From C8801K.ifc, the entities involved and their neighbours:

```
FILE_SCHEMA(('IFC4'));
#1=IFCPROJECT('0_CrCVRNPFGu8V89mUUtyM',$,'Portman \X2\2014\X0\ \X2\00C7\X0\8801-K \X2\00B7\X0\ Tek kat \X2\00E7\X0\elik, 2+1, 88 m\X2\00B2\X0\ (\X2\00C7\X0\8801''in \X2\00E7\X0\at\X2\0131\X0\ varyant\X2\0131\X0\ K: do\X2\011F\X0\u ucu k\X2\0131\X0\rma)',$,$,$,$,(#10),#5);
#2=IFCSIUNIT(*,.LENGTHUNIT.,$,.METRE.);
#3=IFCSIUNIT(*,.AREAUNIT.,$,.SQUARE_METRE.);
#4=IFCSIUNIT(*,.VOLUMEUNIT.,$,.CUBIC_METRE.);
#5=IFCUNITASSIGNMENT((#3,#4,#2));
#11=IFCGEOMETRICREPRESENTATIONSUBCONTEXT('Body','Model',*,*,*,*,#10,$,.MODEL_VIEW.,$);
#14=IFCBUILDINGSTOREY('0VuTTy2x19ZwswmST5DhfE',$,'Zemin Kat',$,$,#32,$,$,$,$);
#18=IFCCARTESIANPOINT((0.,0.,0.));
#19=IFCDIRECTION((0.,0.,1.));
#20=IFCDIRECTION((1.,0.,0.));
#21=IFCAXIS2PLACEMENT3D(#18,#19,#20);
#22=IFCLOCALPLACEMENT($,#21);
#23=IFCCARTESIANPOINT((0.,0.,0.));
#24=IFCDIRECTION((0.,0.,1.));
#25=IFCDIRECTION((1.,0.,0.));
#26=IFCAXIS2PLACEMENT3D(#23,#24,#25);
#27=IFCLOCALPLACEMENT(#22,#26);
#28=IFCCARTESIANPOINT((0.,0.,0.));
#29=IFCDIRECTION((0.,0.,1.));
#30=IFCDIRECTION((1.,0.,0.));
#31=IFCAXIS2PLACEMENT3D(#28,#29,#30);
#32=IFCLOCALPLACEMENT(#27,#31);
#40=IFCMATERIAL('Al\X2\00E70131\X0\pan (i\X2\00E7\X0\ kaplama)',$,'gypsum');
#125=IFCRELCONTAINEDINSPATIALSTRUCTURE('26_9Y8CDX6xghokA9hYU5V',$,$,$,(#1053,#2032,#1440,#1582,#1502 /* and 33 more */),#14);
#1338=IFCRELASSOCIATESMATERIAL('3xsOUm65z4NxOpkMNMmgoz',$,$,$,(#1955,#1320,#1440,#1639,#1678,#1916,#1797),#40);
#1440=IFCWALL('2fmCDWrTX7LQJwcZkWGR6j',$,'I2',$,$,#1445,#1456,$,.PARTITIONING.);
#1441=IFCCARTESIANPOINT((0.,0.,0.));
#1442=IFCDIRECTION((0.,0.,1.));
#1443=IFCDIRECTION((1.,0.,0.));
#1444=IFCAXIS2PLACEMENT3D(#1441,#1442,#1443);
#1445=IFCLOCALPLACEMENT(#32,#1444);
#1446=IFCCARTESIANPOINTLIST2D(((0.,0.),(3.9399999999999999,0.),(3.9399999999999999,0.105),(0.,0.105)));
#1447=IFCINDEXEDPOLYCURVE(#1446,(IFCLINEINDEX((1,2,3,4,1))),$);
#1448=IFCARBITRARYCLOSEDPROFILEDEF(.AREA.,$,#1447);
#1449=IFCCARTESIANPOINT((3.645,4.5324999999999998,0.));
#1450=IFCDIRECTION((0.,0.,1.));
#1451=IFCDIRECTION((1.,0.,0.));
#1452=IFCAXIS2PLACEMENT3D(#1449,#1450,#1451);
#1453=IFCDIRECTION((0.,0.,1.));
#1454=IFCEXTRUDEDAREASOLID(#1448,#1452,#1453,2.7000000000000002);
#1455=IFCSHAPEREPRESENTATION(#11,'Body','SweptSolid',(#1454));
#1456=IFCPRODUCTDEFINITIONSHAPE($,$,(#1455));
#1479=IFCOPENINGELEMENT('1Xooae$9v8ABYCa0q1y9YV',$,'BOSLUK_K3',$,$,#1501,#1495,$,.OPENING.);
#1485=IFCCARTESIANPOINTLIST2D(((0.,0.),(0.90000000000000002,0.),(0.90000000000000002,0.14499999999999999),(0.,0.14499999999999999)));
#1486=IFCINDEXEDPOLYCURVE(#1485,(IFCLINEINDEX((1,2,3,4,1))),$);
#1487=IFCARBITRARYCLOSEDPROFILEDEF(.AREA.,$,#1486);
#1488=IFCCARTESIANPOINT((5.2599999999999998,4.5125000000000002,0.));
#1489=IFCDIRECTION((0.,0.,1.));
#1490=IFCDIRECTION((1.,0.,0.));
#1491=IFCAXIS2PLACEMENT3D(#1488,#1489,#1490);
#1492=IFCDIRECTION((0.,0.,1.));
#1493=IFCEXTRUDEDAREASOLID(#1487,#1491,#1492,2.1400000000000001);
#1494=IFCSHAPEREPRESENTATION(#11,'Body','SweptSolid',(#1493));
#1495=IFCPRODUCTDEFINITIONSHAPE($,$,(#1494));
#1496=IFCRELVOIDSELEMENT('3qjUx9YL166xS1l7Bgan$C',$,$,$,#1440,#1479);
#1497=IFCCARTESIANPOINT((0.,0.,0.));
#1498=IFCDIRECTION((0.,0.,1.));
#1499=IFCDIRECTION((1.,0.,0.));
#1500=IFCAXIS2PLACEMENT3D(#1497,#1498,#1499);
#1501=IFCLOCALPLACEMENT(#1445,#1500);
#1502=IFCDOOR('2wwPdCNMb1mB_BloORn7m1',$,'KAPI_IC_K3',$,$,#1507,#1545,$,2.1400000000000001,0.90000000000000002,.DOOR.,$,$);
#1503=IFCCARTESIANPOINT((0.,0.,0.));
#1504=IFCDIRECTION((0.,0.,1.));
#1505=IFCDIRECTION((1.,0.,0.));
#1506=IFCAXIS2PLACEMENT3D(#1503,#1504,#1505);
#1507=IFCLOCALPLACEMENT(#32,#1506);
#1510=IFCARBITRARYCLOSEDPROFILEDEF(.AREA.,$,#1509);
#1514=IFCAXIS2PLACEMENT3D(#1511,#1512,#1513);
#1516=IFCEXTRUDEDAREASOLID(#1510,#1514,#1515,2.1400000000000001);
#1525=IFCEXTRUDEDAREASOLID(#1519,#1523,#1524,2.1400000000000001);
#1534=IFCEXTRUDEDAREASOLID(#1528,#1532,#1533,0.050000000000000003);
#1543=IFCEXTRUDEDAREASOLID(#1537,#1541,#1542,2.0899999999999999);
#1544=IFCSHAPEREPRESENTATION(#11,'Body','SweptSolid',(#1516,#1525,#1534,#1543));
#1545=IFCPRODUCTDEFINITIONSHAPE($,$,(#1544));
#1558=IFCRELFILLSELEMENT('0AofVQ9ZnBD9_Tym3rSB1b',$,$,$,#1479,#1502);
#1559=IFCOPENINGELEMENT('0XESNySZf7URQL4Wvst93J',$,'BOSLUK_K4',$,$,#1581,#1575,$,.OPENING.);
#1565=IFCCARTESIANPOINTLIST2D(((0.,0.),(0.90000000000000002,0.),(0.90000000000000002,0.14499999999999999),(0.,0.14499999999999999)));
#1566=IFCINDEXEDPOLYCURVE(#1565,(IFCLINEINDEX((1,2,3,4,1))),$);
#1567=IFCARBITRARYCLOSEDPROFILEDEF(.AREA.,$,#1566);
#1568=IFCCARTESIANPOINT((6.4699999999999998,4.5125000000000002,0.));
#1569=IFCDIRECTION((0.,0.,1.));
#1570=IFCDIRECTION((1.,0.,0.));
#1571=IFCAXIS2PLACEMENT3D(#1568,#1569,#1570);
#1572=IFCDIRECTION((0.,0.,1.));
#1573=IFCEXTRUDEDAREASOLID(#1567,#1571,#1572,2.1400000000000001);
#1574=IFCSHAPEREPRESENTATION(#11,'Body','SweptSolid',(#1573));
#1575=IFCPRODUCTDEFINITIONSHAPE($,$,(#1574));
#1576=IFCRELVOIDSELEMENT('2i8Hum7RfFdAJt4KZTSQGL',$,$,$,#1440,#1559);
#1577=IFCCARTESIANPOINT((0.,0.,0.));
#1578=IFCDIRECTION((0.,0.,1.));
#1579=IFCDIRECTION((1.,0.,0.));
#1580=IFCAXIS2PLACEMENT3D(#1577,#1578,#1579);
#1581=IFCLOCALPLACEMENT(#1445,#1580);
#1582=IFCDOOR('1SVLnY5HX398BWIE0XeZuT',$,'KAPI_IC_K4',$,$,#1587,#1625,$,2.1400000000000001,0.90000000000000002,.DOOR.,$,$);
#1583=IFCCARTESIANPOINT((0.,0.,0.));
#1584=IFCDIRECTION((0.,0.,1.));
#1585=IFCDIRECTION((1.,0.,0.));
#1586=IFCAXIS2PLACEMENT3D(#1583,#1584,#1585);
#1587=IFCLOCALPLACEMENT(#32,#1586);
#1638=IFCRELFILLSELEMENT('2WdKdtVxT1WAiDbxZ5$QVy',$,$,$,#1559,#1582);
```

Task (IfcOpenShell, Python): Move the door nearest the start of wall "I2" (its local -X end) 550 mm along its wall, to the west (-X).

```python
import ifcopenshell
import ifcopenshell.api.geometry
import ifcopenshell.util.placement

model = ifcopenshell.open("C8801K.ifc")

door = model.by_id(1502)
opening = door.FillsVoids[0].RelatingOpeningElement
wall = opening.VoidsElements[0].RelatingBuildingElement

wall_matrix = ifcopenshell.util.placement.get_local_placement(wall.ObjectPlacement)
shift = wall_matrix[:3, 0] * -0.55
before = ifcopenshell.util.placement.get_local_placement(door.ObjectPlacement)[:3, 3].copy()

# The door is not placed relative to its opening, so move both.
for product in (opening, door):
    matrix = ifcopenshell.util.placement.get_local_placement(product.ObjectPlacement)
    matrix[:3, 3] += shift
    ifcopenshell.api.geometry.edit_object_placement(model, product=product, matrix=matrix, is_si=False)

after = ifcopenshell.util.placement.get_local_placement(door.ObjectPlacement)[:3, 3]
print("door moved by", (after - before).round(3) + 0.0)

model.write("C8801K_rev.ifc")
```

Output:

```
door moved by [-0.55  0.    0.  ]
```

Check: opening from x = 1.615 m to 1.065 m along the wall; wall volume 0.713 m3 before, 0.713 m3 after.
